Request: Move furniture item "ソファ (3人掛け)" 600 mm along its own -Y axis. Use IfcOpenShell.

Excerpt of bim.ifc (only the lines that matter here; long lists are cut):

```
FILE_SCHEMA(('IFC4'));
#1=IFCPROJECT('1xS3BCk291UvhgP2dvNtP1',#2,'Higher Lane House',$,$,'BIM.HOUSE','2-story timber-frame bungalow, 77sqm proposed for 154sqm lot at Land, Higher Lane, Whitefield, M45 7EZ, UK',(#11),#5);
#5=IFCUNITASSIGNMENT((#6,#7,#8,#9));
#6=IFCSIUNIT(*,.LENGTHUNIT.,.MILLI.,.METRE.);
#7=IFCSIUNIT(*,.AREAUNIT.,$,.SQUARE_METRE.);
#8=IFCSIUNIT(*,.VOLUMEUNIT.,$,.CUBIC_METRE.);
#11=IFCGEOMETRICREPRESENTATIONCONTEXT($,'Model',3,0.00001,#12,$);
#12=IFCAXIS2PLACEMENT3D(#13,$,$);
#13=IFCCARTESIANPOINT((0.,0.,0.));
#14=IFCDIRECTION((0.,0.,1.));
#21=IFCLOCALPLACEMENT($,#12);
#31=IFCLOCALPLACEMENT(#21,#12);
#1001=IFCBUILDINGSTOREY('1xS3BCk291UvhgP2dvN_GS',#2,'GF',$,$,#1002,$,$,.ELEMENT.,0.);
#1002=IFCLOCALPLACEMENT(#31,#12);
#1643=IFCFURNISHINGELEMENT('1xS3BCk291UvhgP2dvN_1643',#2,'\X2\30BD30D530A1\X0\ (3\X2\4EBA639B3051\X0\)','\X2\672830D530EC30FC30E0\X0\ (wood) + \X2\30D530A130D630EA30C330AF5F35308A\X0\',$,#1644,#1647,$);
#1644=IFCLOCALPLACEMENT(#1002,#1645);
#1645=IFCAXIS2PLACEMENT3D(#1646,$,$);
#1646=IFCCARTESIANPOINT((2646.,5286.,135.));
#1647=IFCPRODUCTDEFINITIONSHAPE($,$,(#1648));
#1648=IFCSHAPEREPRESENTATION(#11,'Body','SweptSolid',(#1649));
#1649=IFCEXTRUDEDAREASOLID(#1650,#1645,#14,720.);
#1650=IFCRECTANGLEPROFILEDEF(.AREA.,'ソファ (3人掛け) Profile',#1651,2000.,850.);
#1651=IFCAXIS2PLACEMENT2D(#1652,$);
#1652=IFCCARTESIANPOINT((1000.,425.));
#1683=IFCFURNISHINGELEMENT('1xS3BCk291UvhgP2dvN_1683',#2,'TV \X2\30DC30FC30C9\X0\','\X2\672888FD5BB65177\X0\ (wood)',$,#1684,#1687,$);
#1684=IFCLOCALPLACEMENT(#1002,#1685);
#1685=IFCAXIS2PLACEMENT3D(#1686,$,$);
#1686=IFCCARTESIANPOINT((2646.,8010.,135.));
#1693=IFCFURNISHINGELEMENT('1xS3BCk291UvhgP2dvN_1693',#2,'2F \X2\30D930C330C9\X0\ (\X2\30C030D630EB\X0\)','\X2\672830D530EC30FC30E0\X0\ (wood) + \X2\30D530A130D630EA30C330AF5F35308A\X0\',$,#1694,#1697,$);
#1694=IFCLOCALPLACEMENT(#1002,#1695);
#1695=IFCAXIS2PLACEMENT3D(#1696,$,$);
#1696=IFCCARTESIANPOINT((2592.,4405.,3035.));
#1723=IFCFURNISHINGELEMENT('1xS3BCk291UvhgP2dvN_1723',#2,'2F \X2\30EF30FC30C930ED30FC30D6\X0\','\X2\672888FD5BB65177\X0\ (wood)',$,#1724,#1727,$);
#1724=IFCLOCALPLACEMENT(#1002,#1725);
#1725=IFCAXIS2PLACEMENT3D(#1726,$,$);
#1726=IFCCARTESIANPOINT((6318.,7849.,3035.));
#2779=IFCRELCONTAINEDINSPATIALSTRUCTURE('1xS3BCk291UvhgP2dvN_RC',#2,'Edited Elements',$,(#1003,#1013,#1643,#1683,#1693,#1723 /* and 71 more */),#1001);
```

```python
import ifcopenshell
import ifcopenshell.api.geometry
import ifcopenshell.util.placement
import ifcopenshell.util.unit

model = ifcopenshell.open("bim.ifc")
unit_scale = ifcopenshell.util.unit.calculate_unit_scale(model)

item = model.by_guid("1xS3BCk291UvhgP2dvN_1643")
matrix = ifcopenshell.util.placement.get_local_placement(item.ObjectPlacement)
matrix[:3, 3] -= matrix[:3, 1] * 0.6 / unit_scale
ifcopenshell.api.geometry.edit_object_placement(model, product=item, matrix=matrix, is_si=False)

print(ifcopenshell.util.placement.get_local_placement(item.ObjectPlacement).round(3) + 0.0)

model.write("bim_updated.ifc")
```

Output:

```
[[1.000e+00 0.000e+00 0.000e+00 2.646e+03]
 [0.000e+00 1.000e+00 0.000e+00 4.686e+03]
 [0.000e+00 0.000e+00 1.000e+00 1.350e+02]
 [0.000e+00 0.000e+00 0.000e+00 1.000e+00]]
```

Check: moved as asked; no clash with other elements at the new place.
